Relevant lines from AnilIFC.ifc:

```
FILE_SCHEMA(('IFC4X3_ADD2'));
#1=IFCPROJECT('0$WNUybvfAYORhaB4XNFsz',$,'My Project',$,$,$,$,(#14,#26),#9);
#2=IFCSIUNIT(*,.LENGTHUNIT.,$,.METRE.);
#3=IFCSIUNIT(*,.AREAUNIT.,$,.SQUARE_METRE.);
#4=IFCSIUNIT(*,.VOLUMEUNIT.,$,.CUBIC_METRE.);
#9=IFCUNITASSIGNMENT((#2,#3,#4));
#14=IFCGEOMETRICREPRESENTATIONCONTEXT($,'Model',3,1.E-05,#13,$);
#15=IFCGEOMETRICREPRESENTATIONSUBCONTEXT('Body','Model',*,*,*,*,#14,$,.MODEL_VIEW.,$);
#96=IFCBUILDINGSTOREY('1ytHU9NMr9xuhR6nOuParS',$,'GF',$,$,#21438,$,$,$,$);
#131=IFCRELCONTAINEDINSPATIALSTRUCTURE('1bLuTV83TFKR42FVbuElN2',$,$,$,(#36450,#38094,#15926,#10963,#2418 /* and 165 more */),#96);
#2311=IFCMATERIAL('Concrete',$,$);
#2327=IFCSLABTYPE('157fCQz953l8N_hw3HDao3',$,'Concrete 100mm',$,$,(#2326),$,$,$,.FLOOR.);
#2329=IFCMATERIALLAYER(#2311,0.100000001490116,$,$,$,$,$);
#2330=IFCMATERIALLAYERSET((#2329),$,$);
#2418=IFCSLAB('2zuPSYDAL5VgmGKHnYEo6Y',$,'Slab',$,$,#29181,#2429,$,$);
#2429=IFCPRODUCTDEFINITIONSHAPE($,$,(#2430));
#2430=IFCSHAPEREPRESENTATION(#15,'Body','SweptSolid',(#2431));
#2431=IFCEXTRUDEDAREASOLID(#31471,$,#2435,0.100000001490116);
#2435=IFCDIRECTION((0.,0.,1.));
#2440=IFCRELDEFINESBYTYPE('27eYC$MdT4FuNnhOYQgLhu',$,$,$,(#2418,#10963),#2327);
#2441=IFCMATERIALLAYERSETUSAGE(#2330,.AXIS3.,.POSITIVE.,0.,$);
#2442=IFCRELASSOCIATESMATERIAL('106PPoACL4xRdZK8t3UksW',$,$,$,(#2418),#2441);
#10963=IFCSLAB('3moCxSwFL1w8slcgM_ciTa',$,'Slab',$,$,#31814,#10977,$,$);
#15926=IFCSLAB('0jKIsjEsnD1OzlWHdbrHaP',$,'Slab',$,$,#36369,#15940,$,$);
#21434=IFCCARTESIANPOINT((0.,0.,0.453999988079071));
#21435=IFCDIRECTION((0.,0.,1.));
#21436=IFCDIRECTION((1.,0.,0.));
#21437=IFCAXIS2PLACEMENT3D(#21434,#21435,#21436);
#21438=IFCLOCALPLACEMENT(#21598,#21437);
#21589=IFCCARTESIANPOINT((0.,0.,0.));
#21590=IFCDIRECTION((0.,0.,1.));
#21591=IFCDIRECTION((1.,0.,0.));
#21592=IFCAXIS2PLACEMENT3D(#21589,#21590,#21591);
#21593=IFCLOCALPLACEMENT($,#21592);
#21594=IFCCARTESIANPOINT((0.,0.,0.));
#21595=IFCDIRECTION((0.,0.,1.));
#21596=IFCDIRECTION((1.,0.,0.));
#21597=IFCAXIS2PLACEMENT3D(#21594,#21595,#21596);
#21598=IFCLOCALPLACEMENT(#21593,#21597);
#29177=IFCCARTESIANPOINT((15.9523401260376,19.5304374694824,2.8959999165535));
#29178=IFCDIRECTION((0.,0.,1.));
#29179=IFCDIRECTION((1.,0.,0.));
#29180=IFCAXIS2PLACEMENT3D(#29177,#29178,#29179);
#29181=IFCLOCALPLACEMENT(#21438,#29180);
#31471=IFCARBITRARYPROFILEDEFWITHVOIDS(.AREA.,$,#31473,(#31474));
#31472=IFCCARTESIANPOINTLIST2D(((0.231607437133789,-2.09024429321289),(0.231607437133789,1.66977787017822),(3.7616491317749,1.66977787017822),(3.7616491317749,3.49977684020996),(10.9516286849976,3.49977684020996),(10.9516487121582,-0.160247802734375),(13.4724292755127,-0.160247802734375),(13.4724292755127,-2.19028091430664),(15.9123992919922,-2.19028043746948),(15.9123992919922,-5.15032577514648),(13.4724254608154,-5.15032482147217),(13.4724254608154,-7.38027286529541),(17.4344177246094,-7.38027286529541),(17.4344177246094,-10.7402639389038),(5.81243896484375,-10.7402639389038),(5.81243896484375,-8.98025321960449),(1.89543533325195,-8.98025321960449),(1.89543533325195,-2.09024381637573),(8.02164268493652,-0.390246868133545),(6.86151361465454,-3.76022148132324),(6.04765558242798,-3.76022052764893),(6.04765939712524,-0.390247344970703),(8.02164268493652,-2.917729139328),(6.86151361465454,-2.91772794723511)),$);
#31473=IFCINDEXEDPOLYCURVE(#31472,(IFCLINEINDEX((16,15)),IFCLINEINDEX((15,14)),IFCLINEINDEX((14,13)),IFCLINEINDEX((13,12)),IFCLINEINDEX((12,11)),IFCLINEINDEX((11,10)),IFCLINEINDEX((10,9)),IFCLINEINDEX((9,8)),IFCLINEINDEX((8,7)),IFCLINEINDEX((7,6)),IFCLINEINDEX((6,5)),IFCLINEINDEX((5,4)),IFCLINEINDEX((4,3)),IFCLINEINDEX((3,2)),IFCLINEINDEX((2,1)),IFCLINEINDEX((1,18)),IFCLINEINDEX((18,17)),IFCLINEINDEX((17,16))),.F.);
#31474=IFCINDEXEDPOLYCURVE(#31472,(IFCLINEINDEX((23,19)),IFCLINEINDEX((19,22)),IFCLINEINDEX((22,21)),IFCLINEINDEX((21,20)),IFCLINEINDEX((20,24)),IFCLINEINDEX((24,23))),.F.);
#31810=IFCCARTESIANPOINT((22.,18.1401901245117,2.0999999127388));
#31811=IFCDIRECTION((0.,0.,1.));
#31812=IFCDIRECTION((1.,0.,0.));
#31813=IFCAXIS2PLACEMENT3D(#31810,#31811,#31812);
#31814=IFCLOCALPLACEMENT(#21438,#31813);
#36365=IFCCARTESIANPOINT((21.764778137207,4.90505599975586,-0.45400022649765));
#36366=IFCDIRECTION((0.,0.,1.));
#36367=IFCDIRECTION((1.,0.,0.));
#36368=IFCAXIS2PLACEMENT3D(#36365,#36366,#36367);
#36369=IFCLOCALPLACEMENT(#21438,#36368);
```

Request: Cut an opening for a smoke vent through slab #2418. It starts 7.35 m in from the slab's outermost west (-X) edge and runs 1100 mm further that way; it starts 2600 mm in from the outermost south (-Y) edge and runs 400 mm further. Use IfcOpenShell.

```python
import numpy as np
import ifcopenshell
import ifcopenshell.api.feature
import ifcopenshell.api.geometry
import ifcopenshell.api.root
import ifcopenshell.geom
import ifcopenshell.util.placement
import ifcopenshell.util.representation
import ifcopenshell.util.shape
import ifcopenshell.util.unit

model = ifcopenshell.open("AnilIFC.ifc")
unit_scale = ifcopenshell.util.unit.calculate_unit_scale(model)
settings = ifcopenshell.geom.settings()


def volume(element):
    """Net volume in cubic metres, openings subtracted."""
    shape = ifcopenshell.geom.create_shape(settings, element)
    return ifcopenshell.util.shape.get_volume(shape.geometry)


slab = model.by_guid("2zuPSYDAL5VgmGKHnYEo6Y")
before = volume(slab)

# Extent in the slab's own axes, in metres. The edges named are its -X and -Y sides.
slab_shape = ifcopenshell.geom.create_shape(settings, slab)
vertices = ifcopenshell.util.shape.get_vertices(slab_shape.geometry)
x_min, y_min, bottom = vertices.min(axis=0)
top = vertices[:, 2].max()

opening = ifcopenshell.api.root.create_entity(model, ifc_class="IfcOpeningElement", name="Smoke vent opening", predefined_type="OPENING")
context = ifcopenshell.util.representation.get_context(model, "Model", "Body", "MODEL_VIEW")
width, depth = 1.1, 0.4
outline = [(0.0, 0.0), (width, 0.0), (width, depth), (0.0, depth), (0.0, 0.0)]
# Overshoot both faces by 50 mm so the cut is clean.
shape = ifcopenshell.api.geometry.add_slab_representation(
    model, context=context, depth=top - bottom + 0.1, polyline=outline
)
ifcopenshell.api.geometry.assign_representation(model, product=opening, representation=shape)

matrix = ifcopenshell.util.placement.get_local_placement(slab.ObjectPlacement)
matrix[:, 3] = matrix @ np.append(np.array([x_min + 7.35, y_min + 2.6, bottom - 0.05]) / unit_scale, 1.0)
ifcopenshell.api.geometry.edit_object_placement(model, product=opening, matrix=matrix, is_si=False)
ifcopenshell.api.feature.add_feature(model, feature=opening, element=slab)

after = volume(slab)

print(f"slab volume {before:.3f} -> {after:.3f} m3")

model.write("AnilIFC-out.ifc")
```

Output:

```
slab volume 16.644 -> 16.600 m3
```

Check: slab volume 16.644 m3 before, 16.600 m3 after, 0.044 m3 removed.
